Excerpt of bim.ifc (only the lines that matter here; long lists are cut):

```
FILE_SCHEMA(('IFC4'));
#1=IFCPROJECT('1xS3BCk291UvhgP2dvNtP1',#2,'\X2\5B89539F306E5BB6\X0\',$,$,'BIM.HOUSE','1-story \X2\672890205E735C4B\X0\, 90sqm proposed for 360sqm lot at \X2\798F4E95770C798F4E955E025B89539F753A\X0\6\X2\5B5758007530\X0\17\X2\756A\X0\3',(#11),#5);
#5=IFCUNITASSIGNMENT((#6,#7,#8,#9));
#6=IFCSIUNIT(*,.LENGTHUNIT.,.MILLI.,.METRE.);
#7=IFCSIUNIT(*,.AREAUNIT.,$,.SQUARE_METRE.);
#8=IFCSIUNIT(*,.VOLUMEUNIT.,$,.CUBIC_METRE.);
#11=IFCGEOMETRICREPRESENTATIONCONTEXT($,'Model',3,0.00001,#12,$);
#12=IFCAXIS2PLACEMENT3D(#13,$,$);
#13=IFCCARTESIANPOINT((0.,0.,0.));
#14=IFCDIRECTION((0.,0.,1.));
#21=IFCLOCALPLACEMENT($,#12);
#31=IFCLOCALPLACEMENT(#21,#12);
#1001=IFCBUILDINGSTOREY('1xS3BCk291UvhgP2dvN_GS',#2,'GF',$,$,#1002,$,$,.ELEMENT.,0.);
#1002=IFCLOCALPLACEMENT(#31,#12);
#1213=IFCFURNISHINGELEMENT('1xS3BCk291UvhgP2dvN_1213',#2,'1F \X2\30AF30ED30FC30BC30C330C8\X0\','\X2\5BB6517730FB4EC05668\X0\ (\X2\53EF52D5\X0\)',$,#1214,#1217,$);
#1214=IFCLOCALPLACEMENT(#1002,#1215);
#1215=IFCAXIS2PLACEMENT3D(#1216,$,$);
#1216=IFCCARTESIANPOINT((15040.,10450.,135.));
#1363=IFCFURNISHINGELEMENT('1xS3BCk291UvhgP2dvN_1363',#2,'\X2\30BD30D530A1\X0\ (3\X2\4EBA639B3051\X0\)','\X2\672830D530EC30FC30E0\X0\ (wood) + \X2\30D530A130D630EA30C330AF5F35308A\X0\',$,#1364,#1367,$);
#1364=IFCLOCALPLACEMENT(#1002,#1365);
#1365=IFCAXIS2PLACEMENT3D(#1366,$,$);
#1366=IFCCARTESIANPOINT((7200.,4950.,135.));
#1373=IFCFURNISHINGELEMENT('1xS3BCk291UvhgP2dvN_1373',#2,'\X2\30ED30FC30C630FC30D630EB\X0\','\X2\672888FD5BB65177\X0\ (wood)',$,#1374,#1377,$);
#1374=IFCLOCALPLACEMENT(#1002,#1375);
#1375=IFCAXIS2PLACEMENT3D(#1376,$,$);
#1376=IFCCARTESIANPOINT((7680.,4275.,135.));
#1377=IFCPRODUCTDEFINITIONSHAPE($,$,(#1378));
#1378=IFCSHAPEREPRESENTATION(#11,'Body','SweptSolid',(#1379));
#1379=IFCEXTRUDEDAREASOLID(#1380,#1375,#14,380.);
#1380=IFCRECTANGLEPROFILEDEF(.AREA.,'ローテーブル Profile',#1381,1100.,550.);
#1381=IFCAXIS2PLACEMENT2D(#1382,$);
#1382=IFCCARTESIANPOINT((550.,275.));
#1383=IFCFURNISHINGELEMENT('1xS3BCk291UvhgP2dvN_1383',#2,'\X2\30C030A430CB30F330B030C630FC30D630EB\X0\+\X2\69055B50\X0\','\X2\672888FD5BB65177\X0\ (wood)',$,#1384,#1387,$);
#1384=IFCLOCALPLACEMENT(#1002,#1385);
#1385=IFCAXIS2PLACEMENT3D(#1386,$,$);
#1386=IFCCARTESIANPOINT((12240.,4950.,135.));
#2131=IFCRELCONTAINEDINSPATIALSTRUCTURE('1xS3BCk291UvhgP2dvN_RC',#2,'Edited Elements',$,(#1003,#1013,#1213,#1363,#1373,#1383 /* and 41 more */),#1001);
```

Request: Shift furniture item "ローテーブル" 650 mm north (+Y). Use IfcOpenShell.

```python
import ifcopenshell
import ifcopenshell.api.geometry
import ifcopenshell.util.placement

model = ifcopenshell.open("bim.ifc")

item = model.by_guid("1xS3BCk291UvhgP2dvN_1373")
matrix = ifcopenshell.util.placement.get_local_placement(item.ObjectPlacement)
matrix[1, 3] += 650.0
ifcopenshell.api.geometry.edit_object_placement(model, product=item, matrix=matrix, is_si=False)

print(ifcopenshell.util.placement.get_local_placement(item.ObjectPlacement).round(3) + 0.0)

model.write("bim_rev.ifc")
```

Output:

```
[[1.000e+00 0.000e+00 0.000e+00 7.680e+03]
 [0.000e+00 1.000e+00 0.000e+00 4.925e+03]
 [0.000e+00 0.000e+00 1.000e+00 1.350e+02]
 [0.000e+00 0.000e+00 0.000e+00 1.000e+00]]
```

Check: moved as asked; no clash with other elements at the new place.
